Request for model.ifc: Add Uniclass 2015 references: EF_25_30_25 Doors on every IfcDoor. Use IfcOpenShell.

First a look at what the model holds.

```python
import ifcopenshell

model = ifcopenshell.open("model.ifc")
print(model.schema)
print("classifications:", [c.Name for c in model.by_type("IfcClassification")])
for ifc_class in ("IfcDoor", "IfcRoof", "IfcStair", "IfcWall", "IfcWindow"):
    print(ifc_class, len(model.by_type(ifc_class)))
```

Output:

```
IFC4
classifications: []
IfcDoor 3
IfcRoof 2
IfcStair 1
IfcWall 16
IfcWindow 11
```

```python
import ifcopenshell
import ifcopenshell.api.classification

model = ifcopenshell.open("model.ifc")

system = ifcopenshell.api.classification.add_classification(model, classification="Uniclass 2015")

codes = {
    "IfcDoor": ("EF_25_30_25", "Doors"),
}
for ifc_class, (code, name) in codes.items():
    products = model.by_type(ifc_class)
    ifcopenshell.api.classification.add_reference(
        model, products=products, classification=system, identification=code, name=name
    )
    print(code, len(products))

model.write("model_rev.ifc")
```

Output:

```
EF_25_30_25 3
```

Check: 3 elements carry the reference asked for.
